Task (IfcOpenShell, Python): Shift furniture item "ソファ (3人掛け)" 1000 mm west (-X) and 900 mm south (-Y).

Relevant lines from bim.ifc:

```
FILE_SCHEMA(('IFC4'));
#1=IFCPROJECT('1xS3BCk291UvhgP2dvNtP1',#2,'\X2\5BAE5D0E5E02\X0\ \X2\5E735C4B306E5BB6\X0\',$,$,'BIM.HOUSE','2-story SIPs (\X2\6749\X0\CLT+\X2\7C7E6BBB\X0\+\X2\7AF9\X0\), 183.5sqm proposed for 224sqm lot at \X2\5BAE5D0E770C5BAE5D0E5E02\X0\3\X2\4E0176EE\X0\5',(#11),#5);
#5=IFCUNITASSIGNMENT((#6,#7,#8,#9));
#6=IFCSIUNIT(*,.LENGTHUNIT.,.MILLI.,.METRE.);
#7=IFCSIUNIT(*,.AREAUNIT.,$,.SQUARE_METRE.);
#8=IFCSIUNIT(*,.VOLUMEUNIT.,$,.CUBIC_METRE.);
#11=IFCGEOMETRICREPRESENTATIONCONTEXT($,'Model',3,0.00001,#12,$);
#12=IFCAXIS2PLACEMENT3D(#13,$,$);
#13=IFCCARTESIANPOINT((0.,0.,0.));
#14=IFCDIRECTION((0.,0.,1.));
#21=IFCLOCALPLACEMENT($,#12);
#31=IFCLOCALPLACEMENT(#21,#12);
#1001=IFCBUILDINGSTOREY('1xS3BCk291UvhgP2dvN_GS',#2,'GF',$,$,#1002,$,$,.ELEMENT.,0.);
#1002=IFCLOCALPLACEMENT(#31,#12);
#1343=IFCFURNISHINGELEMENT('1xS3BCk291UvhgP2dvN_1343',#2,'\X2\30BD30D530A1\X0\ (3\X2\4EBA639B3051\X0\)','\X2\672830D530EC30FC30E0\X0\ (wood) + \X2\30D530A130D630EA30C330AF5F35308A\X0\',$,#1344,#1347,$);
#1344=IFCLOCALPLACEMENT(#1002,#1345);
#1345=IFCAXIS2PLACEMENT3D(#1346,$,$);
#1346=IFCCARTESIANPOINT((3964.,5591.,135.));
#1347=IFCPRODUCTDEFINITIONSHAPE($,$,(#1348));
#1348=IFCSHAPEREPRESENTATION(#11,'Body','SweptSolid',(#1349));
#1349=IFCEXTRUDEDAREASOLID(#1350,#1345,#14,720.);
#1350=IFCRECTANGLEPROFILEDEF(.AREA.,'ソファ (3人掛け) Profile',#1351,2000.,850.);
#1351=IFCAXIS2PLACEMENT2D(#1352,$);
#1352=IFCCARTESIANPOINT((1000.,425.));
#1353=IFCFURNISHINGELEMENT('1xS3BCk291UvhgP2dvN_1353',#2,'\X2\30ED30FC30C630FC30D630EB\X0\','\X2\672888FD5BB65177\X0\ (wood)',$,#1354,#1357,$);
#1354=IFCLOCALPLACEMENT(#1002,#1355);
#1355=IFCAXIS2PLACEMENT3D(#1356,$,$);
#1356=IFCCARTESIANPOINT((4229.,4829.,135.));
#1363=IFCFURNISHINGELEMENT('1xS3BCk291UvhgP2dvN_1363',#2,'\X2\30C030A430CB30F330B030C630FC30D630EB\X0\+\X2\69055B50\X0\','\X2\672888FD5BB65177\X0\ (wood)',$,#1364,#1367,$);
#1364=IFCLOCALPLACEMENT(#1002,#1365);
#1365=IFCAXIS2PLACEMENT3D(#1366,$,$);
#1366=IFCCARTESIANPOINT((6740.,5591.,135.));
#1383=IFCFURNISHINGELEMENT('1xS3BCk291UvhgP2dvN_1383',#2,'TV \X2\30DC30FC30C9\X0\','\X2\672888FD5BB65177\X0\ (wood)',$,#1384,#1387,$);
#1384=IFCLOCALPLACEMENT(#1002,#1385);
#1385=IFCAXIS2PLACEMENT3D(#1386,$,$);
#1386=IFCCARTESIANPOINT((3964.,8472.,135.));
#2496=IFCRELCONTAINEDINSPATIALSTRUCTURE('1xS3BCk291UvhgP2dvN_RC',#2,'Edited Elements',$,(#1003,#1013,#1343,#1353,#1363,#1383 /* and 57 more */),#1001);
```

```python
import ifcopenshell
import ifcopenshell.api.geometry
import ifcopenshell.util.placement

model = ifcopenshell.open("bim.ifc")

item = model.by_guid("1xS3BCk291UvhgP2dvN_1343")
matrix = ifcopenshell.util.placement.get_local_placement(item.ObjectPlacement)
matrix[0, 3] -= 1000.0
matrix[1, 3] -= 900.0
ifcopenshell.api.geometry.edit_object_placement(model, product=item, matrix=matrix, is_si=False)

print(ifcopenshell.util.placement.get_local_placement(item.ObjectPlacement).round(3) + 0.0)

model.write("bim_v2.ifc")
```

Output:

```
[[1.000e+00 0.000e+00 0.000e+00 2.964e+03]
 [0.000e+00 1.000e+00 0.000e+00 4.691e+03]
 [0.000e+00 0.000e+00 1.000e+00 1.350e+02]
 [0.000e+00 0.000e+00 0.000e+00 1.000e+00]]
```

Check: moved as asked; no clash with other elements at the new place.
